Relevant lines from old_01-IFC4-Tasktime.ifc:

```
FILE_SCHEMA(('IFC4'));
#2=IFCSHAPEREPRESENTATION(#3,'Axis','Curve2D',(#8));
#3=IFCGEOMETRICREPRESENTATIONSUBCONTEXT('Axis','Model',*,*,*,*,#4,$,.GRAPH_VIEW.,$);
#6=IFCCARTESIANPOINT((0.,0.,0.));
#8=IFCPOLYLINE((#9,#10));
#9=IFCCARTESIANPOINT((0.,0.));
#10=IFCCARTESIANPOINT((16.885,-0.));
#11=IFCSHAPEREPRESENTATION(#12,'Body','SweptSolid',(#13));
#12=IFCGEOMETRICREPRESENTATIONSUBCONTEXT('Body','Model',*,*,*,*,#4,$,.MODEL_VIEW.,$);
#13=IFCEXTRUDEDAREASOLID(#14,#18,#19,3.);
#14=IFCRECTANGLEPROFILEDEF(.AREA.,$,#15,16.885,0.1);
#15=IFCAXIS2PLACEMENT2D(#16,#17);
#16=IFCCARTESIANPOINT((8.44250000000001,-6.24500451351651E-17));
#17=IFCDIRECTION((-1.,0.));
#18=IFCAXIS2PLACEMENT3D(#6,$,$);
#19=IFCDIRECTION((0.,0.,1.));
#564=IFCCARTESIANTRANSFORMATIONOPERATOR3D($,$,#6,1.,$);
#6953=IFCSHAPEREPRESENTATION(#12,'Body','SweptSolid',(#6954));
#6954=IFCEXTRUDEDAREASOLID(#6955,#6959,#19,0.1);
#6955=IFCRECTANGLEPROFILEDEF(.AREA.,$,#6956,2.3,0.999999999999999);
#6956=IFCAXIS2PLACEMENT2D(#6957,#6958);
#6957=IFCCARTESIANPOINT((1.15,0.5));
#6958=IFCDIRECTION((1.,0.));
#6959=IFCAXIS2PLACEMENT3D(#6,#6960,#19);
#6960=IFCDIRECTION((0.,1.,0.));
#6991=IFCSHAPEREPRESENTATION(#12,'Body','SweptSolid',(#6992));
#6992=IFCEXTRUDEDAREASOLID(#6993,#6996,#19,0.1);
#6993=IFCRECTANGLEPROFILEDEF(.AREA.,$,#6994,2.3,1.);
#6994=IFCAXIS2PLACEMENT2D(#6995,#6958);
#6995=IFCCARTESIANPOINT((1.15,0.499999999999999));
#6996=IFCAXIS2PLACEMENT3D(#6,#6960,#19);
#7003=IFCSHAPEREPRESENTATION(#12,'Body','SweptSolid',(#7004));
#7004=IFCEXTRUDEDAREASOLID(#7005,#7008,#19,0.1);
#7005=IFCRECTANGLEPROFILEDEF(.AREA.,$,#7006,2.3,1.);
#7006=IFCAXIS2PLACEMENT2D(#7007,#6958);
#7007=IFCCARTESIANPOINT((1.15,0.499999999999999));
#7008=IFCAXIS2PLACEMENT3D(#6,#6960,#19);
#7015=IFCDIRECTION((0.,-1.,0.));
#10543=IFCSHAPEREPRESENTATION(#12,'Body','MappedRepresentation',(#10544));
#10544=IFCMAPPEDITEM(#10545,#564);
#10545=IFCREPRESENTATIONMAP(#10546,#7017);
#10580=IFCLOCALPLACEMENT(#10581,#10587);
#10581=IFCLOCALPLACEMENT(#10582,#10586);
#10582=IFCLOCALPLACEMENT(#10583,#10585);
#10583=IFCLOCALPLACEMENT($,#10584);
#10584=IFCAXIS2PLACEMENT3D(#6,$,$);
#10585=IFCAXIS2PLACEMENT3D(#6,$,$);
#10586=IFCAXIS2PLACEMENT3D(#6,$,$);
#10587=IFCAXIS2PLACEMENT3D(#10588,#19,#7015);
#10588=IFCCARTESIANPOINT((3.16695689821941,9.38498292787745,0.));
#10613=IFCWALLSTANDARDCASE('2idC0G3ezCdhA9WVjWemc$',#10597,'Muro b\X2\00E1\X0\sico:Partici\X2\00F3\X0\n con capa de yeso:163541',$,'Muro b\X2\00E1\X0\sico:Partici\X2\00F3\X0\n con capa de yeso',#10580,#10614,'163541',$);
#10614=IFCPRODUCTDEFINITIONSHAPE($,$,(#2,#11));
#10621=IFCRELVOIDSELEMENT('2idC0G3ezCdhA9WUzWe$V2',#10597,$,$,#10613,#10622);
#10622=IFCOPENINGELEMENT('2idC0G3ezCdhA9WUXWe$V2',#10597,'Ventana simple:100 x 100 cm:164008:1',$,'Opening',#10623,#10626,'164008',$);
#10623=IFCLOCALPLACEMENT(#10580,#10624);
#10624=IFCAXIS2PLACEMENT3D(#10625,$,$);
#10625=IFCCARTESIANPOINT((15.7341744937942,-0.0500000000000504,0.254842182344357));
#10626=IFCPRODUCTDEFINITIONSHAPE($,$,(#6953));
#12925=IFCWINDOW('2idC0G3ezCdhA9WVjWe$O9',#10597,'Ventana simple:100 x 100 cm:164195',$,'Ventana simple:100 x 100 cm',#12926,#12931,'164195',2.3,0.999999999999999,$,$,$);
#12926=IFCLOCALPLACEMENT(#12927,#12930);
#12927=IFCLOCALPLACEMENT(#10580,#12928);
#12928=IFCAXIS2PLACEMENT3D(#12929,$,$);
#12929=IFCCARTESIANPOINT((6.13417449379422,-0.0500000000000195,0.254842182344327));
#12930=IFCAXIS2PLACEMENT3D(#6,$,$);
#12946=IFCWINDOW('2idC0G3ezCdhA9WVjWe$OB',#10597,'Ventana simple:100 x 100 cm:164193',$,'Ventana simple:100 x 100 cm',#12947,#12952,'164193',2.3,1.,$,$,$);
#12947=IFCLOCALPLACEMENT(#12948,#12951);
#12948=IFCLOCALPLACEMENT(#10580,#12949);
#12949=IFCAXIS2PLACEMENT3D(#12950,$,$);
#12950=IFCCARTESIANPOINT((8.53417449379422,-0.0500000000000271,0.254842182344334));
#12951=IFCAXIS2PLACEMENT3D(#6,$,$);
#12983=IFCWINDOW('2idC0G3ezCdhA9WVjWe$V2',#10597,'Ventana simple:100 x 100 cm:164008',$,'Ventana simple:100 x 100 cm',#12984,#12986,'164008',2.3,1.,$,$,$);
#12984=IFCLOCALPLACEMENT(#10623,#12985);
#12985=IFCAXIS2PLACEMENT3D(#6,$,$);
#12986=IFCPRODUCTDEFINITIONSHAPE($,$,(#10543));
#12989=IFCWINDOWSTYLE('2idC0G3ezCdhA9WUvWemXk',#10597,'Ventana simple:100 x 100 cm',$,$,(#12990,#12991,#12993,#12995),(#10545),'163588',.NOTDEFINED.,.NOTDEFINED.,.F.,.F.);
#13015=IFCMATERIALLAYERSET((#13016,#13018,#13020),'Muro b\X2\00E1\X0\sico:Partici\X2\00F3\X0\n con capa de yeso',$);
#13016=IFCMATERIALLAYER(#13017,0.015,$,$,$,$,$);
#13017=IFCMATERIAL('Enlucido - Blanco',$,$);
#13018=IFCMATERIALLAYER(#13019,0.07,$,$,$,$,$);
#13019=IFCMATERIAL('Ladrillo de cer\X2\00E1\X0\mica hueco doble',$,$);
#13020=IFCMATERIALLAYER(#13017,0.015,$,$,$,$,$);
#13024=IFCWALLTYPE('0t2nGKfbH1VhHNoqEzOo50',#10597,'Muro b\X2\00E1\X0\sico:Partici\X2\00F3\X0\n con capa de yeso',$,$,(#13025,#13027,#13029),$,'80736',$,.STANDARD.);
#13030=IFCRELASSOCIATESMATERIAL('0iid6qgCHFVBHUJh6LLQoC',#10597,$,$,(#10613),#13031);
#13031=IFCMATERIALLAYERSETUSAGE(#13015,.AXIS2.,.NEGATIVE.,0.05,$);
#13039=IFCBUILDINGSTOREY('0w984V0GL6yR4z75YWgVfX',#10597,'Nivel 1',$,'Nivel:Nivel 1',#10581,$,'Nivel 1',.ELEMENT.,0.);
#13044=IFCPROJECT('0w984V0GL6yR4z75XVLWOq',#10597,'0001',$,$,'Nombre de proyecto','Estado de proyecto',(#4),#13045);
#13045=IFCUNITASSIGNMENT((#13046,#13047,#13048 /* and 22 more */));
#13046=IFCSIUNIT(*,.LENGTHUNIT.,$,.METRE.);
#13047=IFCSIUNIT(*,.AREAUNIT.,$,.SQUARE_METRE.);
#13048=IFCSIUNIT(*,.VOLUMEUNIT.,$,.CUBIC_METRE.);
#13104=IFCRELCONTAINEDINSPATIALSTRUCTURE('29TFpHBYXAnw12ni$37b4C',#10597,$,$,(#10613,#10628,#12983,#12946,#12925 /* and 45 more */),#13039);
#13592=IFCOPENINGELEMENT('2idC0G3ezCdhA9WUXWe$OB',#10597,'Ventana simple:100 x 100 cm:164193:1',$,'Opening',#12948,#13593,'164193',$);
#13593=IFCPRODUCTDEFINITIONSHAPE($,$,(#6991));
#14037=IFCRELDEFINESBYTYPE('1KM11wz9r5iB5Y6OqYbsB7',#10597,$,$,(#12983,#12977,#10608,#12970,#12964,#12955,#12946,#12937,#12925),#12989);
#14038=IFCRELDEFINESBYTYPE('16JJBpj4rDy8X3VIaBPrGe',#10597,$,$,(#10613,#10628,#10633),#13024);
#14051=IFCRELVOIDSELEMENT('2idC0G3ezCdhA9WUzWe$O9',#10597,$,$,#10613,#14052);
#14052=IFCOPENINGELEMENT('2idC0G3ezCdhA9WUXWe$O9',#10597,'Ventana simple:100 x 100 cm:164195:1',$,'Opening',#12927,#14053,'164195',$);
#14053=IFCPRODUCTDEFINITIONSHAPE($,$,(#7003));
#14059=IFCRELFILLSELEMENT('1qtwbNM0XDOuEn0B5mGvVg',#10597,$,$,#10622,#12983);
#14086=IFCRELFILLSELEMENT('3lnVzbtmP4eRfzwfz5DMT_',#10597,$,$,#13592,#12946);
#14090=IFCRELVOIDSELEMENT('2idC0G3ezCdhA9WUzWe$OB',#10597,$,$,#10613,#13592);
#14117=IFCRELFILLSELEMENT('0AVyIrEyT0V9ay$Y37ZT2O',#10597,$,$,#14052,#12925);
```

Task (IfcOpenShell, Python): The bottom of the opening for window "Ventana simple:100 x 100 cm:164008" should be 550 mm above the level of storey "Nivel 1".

```python
import numpy as np
import ifcopenshell
import ifcopenshell.api.geometry
import ifcopenshell.geom
import ifcopenshell.util.element
import ifcopenshell.util.placement
import ifcopenshell.util.shape
import ifcopenshell.util.unit

model = ifcopenshell.open("old_01-IFC4-Tasktime.ifc")
unit_scale = ifcopenshell.util.unit.calculate_unit_scale(model)

window = model.by_guid("2idC0G3ezCdhA9WVjWe$V2")
opening = window.FillsVoids[0].RelatingOpeningElement
storey = ifcopenshell.util.element.get_container(window, ifc_class="IfcBuildingStorey")
level = ifcopenshell.util.placement.get_local_placement(storey.ObjectPlacement)[2, 3]

# The opening's origin need not be at the sill, so measure its lowest point.
shape = ifcopenshell.geom.create_shape(ifcopenshell.geom.settings(), opening)
bottom = ifcopenshell.util.shape.get_shape_bottom_elevation(shape, shape.geometry) / unit_scale
dz = level + 0.55 - bottom

shift = np.array([0.0, 0.0, dz])
# The window is placed relative to its opening, so it follows when the opening moves.
matrix = ifcopenshell.util.placement.get_local_placement(opening.ObjectPlacement)
matrix[:3, 3] += shift
ifcopenshell.api.geometry.edit_object_placement(
    model, product=opening, matrix=matrix, is_si=False, should_transform_children=True
)

print(f"moved by {dz * unit_scale:+.3f} m")

model.write("old_01-IFC4-Tasktime_rev.ifc")
```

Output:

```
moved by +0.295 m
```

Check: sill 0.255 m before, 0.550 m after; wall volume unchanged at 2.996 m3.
